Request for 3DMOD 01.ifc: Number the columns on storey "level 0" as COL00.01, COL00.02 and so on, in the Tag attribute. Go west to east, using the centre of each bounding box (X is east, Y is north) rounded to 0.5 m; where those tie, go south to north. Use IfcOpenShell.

First a look at what the model holds.

```python
import ifcopenshell
import ifcopenshell.util.element
import ifcopenshell.util.placement

model = ifcopenshell.open("3DMOD 01.ifc")
print(model.schema)
storey = next(s for s in model.by_type("IfcBuildingStorey") if s.Name == "level 0")
columns = [e for e in ifcopenshell.util.element.get_decomposition(storey) if e.is_a("IfcColumn")]
for e in sorted(columns, key=lambda e: e.id()):
    origin = ifcopenshell.util.placement.get_local_placement(e.ObjectPlacement)[:3, 3]
    print(e.id(), e.Tag, e.Name, origin.round(2) + 0.0, sep=" | ")
```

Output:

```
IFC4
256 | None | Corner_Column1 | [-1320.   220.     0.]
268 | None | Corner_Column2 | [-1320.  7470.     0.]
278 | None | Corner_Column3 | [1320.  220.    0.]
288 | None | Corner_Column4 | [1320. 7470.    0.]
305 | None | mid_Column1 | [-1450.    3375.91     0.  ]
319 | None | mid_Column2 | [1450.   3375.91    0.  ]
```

```python
import ifcopenshell
import ifcopenshell.geom
import ifcopenshell.util.element
import ifcopenshell.util.shape

model = ifcopenshell.open("3DMOD 01.ifc")
settings = ifcopenshell.geom.settings()
settings.set("use-world-coords", True)


def centre(element):
    shape = ifcopenshell.geom.create_shape(settings, element)
    return ifcopenshell.util.shape.get_bbox_centroid(shape.geometry)


storey = next(s for s in model.by_type("IfcBuildingStorey") if s.Name == "level 0")
columns = [e for e in ifcopenshell.util.element.get_decomposition(storey) if e.is_a("IfcColumn")]

# Insertion points can sit at a corner or the storey origin, so sort by the geometry (in metres).
centres = {e: centre(e) for e in columns}
columns.sort(key=lambda e: (round(centres[e][0] / 0.5), centres[e][1]))

for i, e in enumerate(columns, start=1):
    number = f"COL00.{i:02d}"
    e.Tag = number
    print(e.id(), number)

model.write("3DMOD 01-out.ifc")
```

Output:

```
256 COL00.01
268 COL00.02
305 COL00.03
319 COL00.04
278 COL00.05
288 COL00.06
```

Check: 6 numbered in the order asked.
